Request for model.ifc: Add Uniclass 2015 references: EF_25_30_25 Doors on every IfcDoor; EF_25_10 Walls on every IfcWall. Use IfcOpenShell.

First a look at what the model holds.

```python
import ifcopenshell

model = ifcopenshell.open("model.ifc")
print(model.schema)
print("classifications:", [c.Name for c in model.by_type("IfcClassification")])
for ifc_class in ("IfcDoor", "IfcRoof", "IfcStair", "IfcWall", "IfcWindow"):
    print(ifc_class, len(model.by_type(ifc_class)))
```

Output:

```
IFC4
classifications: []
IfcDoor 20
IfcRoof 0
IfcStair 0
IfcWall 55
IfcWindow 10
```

```python
import ifcopenshell
import ifcopenshell.api.classification

model = ifcopenshell.open("model.ifc")

system = ifcopenshell.api.classification.add_classification(model, classification="Uniclass 2015")

codes = {
    "IfcDoor": ("EF_25_30_25", "Doors"),
    "IfcWall": ("EF_25_10", "Walls"),
}
for ifc_class, (code, name) in codes.items():
    products = model.by_type(ifc_class)
    ifcopenshell.api.classification.add_reference(
        model, products=products, classification=system, identification=code, name=name
    )
    print(code, len(products))

model.write("model_v2.ifc")
```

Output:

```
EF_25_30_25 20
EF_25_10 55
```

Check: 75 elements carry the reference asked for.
